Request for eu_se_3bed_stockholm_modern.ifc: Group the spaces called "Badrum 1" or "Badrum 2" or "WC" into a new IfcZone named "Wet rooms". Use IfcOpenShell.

First a look at what the model holds.

```python
import ifcopenshell

model = ifcopenshell.open("eu_se_3bed_stockholm_modern.ifc")
print(model.schema)
seen = {}
for space in model.by_type("IfcSpace"):
    seen[space.LongName] = seen.get(space.LongName, 0) + 1
for name, count in sorted(seen.items(), key=str):
    print(count, "x", name)
print("zones:", [z.Name for z in model.by_type("IfcZone")][:20])
```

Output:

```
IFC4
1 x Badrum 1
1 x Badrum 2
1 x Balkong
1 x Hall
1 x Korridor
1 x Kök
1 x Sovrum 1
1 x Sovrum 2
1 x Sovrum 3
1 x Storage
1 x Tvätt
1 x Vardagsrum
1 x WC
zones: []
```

```python
import ifcopenshell
import ifcopenshell.api.group
import ifcopenshell.api.root

model = ifcopenshell.open("eu_se_3bed_stockholm_modern.ifc")

names = {"Badrum 1", "Badrum 2", "WC"}
spaces = [s for s in model.by_type("IfcSpace") if s.LongName in names]

zone = ifcopenshell.api.root.create_entity(model, ifc_class="IfcZone", name="Wet rooms")
ifcopenshell.api.group.assign_group(model, products=spaces, group=zone)
print(len(spaces), "spaces in", zone.Name)

model.write("eu_se_3bed_stockholm_modern_rev.ifc")
```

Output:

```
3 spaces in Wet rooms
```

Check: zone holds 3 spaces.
